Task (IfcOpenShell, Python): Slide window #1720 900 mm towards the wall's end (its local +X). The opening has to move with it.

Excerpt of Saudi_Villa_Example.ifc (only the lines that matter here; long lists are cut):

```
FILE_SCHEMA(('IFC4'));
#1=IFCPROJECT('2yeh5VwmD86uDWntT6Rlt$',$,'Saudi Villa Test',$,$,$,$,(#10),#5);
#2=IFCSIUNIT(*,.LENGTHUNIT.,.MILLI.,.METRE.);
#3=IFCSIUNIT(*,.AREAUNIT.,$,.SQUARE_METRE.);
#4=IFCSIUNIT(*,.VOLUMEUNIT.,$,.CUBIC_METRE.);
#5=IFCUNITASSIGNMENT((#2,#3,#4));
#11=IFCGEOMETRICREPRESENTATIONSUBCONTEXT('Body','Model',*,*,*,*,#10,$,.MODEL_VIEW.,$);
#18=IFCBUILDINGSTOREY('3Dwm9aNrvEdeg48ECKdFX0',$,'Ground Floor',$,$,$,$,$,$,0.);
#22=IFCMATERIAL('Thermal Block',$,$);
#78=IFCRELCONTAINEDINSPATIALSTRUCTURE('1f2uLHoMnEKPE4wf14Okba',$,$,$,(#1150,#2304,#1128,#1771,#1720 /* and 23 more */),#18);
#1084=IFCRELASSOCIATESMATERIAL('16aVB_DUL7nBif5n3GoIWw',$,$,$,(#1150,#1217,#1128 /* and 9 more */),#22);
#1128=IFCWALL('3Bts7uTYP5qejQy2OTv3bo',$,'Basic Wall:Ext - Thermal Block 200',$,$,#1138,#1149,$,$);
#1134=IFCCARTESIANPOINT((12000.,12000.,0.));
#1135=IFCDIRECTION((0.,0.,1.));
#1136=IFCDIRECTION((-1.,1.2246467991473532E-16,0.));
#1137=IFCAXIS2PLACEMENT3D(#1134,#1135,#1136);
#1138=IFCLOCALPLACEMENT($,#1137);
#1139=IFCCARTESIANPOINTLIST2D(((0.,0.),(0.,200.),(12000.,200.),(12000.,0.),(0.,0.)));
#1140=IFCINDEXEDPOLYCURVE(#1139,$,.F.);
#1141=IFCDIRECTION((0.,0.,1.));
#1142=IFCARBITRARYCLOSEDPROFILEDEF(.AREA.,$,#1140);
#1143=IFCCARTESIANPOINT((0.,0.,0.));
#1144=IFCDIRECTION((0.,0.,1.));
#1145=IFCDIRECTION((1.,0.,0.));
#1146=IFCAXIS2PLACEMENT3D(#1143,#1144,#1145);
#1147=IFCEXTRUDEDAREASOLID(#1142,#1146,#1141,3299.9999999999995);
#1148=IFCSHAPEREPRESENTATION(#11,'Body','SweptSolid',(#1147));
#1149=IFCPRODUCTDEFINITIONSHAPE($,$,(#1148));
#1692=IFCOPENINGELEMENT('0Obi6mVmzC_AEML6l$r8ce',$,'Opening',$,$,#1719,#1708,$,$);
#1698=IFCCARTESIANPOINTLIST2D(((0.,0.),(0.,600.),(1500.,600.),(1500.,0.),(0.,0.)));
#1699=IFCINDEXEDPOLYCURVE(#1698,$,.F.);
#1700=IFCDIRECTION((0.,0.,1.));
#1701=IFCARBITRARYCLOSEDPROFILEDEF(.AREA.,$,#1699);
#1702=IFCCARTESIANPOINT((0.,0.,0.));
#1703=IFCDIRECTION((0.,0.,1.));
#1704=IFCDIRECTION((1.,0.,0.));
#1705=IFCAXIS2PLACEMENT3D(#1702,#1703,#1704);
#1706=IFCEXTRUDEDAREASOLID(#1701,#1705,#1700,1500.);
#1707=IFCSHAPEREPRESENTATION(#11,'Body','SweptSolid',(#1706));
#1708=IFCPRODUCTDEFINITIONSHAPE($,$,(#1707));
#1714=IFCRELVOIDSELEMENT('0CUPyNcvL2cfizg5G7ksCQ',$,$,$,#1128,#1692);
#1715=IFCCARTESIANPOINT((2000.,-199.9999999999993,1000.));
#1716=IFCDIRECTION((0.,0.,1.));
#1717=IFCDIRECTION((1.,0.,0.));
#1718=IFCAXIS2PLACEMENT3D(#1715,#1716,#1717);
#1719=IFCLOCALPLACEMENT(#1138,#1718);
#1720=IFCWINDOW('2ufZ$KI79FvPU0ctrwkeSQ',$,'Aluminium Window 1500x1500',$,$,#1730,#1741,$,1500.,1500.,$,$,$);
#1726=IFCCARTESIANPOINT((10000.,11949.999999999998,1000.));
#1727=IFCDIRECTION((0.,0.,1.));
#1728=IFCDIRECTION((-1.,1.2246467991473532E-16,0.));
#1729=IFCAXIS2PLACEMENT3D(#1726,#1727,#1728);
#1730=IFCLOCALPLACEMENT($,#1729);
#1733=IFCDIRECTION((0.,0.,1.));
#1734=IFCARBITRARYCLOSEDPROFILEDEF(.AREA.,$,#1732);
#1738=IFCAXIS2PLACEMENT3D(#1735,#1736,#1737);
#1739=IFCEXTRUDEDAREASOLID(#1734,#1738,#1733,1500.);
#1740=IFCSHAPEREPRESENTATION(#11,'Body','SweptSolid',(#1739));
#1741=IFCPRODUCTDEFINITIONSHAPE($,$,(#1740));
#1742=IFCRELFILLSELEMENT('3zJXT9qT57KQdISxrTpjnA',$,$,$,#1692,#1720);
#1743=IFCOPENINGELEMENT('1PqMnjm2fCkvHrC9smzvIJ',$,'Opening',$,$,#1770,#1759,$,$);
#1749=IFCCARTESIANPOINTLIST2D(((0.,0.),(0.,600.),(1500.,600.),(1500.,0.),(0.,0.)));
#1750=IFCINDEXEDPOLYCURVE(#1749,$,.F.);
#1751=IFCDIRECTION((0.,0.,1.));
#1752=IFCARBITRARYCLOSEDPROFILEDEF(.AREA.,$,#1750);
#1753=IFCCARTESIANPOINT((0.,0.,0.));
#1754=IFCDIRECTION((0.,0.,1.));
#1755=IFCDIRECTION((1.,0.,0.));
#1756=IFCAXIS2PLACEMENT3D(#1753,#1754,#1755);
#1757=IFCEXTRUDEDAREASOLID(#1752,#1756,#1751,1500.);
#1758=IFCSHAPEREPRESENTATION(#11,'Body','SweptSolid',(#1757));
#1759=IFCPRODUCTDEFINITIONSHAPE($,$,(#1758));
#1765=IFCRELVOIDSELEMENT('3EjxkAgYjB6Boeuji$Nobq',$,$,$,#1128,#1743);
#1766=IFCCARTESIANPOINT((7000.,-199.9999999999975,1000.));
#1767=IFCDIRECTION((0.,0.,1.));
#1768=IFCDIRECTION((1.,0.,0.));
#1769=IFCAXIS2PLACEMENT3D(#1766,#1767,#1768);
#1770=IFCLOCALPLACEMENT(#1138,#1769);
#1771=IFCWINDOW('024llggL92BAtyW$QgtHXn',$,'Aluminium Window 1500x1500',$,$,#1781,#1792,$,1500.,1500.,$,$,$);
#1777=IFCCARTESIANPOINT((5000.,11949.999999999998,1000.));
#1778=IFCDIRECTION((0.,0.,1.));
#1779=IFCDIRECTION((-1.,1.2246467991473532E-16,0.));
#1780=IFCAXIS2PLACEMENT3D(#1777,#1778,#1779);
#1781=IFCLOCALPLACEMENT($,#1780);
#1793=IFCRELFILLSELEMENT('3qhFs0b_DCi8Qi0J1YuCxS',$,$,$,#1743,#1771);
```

```python
import ifcopenshell
import ifcopenshell.api.geometry
import ifcopenshell.util.placement
import ifcopenshell.util.unit

model = ifcopenshell.open("Saudi_Villa_Example.ifc")
unit_scale = ifcopenshell.util.unit.calculate_unit_scale(model)

window = model.by_guid("2ufZ$KI79FvPU0ctrwkeSQ")
opening = window.FillsVoids[0].RelatingOpeningElement
wall = opening.VoidsElements[0].RelatingBuildingElement

wall_matrix = ifcopenshell.util.placement.get_local_placement(wall.ObjectPlacement)
shift = wall_matrix[:3, 0] * 0.9 / unit_scale
before = ifcopenshell.util.placement.get_local_placement(window.ObjectPlacement)[:3, 3].copy()

# The window is not placed relative to its opening, so move both.
for product in (opening, window):
    matrix = ifcopenshell.util.placement.get_local_placement(product.ObjectPlacement)
    matrix[:3, 3] += shift
    ifcopenshell.api.geometry.edit_object_placement(model, product=product, matrix=matrix, is_si=False)

after = ifcopenshell.util.placement.get_local_placement(window.ObjectPlacement)[:3, 3]
print("window moved by", (after - before).round(3) + 0.0)

model.write("Saudi_Villa_Example_edited.ifc")
```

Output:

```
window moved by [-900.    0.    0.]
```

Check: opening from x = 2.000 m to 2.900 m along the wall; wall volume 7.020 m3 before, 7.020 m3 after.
